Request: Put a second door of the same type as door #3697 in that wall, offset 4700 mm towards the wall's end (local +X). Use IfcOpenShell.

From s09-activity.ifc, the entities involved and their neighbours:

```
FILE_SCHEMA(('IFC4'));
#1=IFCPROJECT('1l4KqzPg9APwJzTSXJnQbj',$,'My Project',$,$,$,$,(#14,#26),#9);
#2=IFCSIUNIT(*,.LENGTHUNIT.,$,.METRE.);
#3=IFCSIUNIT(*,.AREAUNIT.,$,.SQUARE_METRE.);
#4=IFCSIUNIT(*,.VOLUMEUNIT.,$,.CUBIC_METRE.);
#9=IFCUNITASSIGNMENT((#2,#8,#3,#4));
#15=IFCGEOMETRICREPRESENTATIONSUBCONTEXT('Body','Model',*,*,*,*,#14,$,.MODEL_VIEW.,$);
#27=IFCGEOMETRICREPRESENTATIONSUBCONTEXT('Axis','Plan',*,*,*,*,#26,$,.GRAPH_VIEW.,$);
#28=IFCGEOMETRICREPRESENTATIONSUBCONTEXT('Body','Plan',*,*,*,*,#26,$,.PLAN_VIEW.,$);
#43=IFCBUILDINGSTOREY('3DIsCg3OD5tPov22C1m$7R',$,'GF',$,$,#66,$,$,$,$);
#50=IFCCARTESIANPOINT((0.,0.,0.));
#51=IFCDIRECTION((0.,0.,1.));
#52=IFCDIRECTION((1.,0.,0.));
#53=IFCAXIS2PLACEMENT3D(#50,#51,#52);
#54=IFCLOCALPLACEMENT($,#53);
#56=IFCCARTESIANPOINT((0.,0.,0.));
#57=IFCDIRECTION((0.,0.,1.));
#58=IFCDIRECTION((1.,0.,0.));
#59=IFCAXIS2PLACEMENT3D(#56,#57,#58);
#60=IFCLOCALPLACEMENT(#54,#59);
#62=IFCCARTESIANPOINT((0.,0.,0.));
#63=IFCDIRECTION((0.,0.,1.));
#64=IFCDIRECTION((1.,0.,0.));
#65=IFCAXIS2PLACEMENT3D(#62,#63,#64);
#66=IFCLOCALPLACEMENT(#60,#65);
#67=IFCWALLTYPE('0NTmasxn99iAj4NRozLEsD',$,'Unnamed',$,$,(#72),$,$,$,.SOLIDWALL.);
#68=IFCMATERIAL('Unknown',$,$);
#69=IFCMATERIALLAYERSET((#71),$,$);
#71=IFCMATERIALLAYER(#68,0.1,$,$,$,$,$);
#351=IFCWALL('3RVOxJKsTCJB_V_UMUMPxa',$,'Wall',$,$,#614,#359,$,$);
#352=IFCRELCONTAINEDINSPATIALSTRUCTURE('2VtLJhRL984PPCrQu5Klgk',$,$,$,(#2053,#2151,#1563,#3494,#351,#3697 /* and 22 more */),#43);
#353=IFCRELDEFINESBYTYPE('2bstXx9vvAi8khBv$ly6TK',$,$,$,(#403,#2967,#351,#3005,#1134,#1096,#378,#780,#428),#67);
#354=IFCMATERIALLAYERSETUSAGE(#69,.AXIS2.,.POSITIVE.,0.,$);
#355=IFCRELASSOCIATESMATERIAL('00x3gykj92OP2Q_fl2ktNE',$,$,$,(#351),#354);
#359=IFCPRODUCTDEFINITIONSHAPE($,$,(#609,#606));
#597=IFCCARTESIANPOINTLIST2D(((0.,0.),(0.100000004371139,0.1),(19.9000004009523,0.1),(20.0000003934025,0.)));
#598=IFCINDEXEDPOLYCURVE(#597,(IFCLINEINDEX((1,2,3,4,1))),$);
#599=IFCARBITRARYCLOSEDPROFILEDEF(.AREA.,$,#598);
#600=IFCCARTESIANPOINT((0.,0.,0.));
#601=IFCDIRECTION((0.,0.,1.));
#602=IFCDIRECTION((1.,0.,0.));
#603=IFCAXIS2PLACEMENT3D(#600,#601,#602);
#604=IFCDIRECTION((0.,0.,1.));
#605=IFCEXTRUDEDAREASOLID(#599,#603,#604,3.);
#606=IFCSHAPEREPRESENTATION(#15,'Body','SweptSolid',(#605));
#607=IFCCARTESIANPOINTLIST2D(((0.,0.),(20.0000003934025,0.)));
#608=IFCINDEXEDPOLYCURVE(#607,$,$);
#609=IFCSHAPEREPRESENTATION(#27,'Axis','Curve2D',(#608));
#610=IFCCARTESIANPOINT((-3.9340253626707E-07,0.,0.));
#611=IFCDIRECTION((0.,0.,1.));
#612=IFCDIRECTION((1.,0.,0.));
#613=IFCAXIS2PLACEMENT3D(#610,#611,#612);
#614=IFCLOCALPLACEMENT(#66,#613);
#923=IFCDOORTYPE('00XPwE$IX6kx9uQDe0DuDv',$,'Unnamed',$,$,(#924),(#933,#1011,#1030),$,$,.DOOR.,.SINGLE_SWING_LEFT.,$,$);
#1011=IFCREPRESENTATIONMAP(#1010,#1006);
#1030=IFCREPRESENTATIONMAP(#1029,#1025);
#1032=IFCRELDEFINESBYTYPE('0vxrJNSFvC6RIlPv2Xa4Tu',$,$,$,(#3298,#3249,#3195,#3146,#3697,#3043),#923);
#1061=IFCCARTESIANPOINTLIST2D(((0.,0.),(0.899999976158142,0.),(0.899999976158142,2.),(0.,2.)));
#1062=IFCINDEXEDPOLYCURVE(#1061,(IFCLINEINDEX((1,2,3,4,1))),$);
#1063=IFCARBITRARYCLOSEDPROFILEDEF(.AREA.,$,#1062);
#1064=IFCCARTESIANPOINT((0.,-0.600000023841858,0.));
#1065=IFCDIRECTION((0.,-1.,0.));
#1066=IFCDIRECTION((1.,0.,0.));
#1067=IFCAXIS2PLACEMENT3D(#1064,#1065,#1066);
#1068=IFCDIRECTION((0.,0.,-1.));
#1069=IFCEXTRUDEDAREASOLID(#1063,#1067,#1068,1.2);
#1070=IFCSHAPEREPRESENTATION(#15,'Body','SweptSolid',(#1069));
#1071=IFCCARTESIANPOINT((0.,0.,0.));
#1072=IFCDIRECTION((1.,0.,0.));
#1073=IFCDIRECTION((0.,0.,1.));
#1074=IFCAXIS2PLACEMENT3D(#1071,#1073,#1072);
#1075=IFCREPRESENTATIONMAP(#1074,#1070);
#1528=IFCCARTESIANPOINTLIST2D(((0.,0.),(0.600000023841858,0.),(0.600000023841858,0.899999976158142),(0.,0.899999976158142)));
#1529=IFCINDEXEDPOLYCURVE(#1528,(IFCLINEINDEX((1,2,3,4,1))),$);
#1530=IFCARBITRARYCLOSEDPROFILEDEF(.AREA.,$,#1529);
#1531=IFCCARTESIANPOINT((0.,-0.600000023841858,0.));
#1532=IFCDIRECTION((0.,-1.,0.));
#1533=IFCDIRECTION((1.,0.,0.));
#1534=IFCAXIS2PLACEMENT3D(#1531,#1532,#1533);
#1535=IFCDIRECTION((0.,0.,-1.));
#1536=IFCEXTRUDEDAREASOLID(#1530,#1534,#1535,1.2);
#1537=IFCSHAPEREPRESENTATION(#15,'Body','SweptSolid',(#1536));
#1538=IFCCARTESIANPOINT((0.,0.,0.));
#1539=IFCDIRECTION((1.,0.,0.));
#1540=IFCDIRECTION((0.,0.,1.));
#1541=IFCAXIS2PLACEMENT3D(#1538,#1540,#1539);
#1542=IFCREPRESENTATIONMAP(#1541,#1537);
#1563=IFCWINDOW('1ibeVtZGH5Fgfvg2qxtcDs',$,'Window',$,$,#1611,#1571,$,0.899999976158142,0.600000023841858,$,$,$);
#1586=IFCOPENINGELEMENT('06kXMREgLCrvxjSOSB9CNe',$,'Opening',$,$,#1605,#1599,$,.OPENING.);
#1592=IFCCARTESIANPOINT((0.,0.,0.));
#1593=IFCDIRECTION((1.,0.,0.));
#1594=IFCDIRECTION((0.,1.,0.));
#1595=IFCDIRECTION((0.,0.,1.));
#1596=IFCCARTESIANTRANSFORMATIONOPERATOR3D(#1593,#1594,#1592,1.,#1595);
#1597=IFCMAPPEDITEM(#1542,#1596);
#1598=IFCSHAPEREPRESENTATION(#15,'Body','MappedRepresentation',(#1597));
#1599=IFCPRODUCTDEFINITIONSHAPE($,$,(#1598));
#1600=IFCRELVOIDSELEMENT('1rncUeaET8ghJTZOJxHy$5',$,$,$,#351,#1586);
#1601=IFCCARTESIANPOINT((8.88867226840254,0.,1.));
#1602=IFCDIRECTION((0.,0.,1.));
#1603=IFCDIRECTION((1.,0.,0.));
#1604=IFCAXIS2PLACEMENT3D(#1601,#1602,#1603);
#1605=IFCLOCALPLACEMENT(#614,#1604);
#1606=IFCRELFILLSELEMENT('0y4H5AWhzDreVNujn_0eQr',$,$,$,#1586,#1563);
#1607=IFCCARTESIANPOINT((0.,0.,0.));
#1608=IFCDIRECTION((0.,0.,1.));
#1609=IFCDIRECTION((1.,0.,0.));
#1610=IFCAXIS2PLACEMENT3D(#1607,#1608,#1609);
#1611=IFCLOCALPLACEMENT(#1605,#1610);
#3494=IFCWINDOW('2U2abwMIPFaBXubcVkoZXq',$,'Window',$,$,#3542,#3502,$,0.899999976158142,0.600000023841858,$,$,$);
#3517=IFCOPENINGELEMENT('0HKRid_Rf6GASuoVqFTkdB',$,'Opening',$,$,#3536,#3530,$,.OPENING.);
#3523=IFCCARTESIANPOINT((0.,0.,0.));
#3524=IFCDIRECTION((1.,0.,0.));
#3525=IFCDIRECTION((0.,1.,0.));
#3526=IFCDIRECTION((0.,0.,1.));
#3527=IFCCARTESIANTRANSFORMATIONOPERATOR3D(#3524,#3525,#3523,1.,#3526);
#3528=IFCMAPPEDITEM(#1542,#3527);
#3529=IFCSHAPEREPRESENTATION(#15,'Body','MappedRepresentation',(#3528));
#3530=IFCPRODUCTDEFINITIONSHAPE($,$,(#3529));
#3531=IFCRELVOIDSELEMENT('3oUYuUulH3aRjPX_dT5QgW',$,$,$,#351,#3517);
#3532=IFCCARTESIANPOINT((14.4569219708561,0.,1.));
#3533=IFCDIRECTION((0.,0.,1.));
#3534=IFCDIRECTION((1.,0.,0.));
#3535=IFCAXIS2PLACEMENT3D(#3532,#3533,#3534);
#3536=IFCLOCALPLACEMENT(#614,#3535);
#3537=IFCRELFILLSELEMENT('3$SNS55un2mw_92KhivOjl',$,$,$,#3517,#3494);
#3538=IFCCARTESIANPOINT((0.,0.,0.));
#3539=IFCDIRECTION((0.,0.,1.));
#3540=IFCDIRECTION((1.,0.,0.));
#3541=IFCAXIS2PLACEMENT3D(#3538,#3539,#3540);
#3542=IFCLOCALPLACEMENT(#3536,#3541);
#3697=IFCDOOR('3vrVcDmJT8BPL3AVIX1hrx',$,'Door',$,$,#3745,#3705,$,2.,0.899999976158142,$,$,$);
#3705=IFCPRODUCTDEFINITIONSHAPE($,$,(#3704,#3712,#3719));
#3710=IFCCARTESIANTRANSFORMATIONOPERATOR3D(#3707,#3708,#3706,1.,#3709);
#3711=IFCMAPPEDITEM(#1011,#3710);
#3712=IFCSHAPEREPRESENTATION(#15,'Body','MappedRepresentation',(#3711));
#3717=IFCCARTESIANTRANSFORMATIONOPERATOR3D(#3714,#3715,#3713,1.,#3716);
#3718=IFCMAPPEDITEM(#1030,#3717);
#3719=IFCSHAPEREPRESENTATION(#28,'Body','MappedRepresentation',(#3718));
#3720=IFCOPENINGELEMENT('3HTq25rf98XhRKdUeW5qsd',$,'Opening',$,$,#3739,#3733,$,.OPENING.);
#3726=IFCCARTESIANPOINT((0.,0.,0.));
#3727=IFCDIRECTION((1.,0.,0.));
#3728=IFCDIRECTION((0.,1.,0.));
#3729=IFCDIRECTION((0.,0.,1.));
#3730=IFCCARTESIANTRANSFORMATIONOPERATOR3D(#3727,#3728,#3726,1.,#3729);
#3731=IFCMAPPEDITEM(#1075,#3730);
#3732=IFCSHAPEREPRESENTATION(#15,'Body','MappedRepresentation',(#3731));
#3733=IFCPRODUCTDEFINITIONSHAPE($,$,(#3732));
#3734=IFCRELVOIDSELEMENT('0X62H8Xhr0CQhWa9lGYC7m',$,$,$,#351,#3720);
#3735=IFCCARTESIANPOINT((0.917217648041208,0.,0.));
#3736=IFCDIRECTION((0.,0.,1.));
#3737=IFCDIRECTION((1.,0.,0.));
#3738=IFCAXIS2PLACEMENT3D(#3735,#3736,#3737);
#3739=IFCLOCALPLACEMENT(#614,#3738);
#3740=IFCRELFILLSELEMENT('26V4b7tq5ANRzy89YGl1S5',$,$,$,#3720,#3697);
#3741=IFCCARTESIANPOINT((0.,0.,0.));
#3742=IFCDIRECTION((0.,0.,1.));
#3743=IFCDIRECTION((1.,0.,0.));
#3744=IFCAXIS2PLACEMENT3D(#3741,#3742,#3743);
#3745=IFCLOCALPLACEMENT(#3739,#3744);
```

```python
import ifcopenshell
import ifcopenshell.api.feature
import ifcopenshell.api.geometry
import ifcopenshell.api.root
import ifcopenshell.geom
import ifcopenshell.util.element
import ifcopenshell.util.placement
import ifcopenshell.util.shape
import ifcopenshell.util.unit

model = ifcopenshell.open("s09-activity.ifc")
unit_scale = ifcopenshell.util.unit.calculate_unit_scale(model)
settings = ifcopenshell.geom.settings()


def volume(element):
    """Net volume in cubic metres, openings subtracted."""
    shape = ifcopenshell.geom.create_shape(settings, element)
    return ifcopenshell.util.shape.get_volume(shape.geometry)


door = model.by_guid("3vrVcDmJT8BPL3AVIX1hrx")
opening = door.FillsVoids[0].RelatingOpeningElement
wall = opening.VoidsElements[0].RelatingBuildingElement
before = volume(wall)
shift = ifcopenshell.util.placement.get_local_placement(wall.ObjectPlacement)[:3, 0] * 4.7 / unit_scale

# copy_class copies the void relationship, type, container and properties, but no geometry.
new_opening = ifcopenshell.api.root.copy_class(model, product=opening)
new_opening.Representation = ifcopenshell.util.element.copy_deep(
    model, opening.Representation, exclude=["IfcGeometricRepresentationContext", "IfcRepresentationMap"]
)
new_door = ifcopenshell.api.root.copy_class(model, product=door)
new_door.Representation = ifcopenshell.util.element.copy_deep(
    model, door.Representation, exclude=["IfcGeometricRepresentationContext", "IfcRepresentationMap"]
)
ifcopenshell.api.feature.add_filling(model, opening=new_opening, element=new_door)

for old, new in ((opening, new_opening), (door, new_door)):
    matrix = ifcopenshell.util.placement.get_local_placement(old.ObjectPlacement)
    matrix[:3, 3] += shift
    ifcopenshell.api.geometry.edit_object_placement(model, product=new, matrix=matrix, is_si=False)

after = volume(wall)

print(f"wall volume {before:.3f} -> {after:.3f} m3")

model.write("s09-activity_edited.ifc")
```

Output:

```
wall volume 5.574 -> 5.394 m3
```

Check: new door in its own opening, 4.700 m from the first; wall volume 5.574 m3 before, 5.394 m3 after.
